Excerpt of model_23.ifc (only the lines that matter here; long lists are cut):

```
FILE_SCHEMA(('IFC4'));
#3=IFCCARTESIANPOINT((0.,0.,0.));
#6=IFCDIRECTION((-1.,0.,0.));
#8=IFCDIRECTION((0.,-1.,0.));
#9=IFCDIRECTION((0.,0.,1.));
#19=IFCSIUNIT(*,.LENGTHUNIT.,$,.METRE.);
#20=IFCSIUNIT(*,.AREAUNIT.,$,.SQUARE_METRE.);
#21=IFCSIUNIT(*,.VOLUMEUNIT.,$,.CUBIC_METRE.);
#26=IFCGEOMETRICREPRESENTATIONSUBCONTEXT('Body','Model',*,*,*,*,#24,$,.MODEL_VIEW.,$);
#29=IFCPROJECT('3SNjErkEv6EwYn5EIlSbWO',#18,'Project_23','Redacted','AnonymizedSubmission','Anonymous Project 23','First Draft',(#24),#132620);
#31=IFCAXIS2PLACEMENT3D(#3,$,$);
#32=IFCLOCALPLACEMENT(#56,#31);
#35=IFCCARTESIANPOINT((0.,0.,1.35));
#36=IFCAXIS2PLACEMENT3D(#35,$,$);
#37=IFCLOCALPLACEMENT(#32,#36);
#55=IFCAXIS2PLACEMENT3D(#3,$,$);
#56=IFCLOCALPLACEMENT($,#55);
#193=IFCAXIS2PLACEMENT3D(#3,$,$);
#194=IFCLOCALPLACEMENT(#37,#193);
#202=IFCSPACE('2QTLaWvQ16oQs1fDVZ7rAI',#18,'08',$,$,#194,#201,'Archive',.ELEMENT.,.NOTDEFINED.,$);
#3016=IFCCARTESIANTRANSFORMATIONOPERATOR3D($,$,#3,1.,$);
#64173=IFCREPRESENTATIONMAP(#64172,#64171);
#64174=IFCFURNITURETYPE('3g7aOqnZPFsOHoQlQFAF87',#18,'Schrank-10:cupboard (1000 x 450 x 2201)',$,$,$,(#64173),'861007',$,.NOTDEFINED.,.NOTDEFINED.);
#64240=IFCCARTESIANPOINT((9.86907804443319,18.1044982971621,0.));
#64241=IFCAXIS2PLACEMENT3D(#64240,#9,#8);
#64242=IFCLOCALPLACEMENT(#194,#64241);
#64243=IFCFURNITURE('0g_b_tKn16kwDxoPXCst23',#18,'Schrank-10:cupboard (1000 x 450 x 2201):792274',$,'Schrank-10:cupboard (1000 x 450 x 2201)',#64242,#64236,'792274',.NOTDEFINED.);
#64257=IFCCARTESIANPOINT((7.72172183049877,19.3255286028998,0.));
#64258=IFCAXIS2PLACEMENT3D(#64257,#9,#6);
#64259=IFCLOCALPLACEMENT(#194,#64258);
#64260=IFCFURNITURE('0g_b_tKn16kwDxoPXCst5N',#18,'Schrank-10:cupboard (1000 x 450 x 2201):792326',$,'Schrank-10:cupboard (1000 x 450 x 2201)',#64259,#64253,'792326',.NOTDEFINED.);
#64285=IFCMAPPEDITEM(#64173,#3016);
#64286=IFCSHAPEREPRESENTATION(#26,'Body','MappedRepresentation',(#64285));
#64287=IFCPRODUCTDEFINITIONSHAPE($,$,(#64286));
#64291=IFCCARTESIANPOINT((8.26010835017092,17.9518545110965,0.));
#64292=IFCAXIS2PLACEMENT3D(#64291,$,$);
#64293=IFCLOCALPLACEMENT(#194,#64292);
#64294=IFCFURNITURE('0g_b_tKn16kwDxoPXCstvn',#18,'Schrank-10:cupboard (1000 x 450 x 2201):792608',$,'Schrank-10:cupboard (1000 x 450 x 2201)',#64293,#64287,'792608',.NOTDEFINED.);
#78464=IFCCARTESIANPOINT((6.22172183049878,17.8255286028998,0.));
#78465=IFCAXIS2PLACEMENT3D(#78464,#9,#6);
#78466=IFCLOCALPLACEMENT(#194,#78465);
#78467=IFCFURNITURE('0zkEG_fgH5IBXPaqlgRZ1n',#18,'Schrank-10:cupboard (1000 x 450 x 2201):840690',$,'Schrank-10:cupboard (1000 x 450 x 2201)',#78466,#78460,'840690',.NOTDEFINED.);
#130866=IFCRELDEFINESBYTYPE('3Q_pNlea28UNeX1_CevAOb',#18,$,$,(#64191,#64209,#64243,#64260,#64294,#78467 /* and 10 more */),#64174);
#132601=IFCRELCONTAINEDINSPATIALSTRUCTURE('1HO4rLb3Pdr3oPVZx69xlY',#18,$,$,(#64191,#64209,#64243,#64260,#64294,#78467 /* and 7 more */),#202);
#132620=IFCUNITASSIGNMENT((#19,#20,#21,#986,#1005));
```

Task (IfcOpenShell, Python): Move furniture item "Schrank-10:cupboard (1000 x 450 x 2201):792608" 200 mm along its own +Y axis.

```python
import ifcopenshell
import ifcopenshell.api.geometry
import ifcopenshell.util.placement
import ifcopenshell.util.unit

model = ifcopenshell.open("model_23.ifc")
unit_scale = ifcopenshell.util.unit.calculate_unit_scale(model)

item = model.by_guid("0g_b_tKn16kwDxoPXCstvn")
matrix = ifcopenshell.util.placement.get_local_placement(item.ObjectPlacement)
matrix[:3, 3] += matrix[:3, 1] * 0.2 / unit_scale
ifcopenshell.api.geometry.edit_object_placement(model, product=item, matrix=matrix, is_si=False)

print(ifcopenshell.util.placement.get_local_placement(item.ObjectPlacement).round(3) + 0.0)

model.write("model_23_updated.ifc")
```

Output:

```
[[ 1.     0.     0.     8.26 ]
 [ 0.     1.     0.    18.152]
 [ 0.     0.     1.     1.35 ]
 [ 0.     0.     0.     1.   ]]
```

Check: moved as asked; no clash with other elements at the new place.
